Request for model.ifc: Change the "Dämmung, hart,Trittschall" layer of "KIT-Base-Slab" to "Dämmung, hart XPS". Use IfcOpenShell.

First a look at what the model holds.

```python
import ifcopenshell
import ifcopenshell.util.element

model = ifcopenshell.open("model.ifc")
print(model.schema)
for layer_set in model.by_type("IfcMaterialLayerSet"):
    if layer_set.LayerSetName == "KIT-Base-Slab":
        for layer in layer_set.MaterialLayers:
            print(layer.id(), layer.Material and layer.Material.Name, layer.LayerThickness, sep=" | ")
        print(len(ifcopenshell.util.element.get_elements_by_material(model, layer_set)), "elements and types use it")
print(sorted(m.Name for m in model.by_type("IfcMaterial") if m.Name)[:60])
```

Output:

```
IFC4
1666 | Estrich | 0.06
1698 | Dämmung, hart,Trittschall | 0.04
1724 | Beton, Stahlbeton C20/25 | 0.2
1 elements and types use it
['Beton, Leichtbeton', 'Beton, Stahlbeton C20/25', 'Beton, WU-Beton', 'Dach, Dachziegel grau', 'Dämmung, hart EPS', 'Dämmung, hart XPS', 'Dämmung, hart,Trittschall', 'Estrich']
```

```python
import ifcopenshell
import ifcopenshell.api.material

model = ifcopenshell.open("model.ifc")

layer_set = next(s for s in model.by_type("IfcMaterialLayerSet") if s.LayerSetName == "KIT-Base-Slab")
layer = next(l for l in layer_set.MaterialLayers if l.Material and l.Material.Name == "Dämmung, hart,Trittschall")
material = next(m for m in model.by_type("IfcMaterial") if m.Name == "Dämmung, hart XPS")

# Point this one layer at the other material; renaming the old one would change it everywhere.
ifcopenshell.api.material.edit_layer(model, layer=layer, attributes={}, material=material)

print([l.Material.Name if l.Material else None for l in layer_set.MaterialLayers])

model.write("model_v2.ifc")
```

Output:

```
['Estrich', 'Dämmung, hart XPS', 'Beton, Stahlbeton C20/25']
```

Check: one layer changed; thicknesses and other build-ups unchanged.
